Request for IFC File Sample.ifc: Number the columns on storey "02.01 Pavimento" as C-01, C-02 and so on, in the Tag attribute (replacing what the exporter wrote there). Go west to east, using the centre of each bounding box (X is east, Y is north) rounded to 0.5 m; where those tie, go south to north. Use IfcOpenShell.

First a look at what the model holds.

```python
import ifcopenshell
import ifcopenshell.util.element
import ifcopenshell.util.placement

model = ifcopenshell.open("IFC File Sample.ifc")
print(model.schema)
storey = next(s for s in model.by_type("IfcBuildingStorey") if s.Name == "02.01 Pavimento")
columns = [e for e in ifcopenshell.util.element.get_decomposition(storey) if e.is_a("IfcColumn")]
for e in sorted(columns, key=lambda e: e.id()):
    origin = ifcopenshell.util.placement.get_local_placement(e.ObjectPlacement)[:3, 3]
    print(e.id(), e.Tag, e.Name, origin.round(2) + 0.0, sep=" | ")
```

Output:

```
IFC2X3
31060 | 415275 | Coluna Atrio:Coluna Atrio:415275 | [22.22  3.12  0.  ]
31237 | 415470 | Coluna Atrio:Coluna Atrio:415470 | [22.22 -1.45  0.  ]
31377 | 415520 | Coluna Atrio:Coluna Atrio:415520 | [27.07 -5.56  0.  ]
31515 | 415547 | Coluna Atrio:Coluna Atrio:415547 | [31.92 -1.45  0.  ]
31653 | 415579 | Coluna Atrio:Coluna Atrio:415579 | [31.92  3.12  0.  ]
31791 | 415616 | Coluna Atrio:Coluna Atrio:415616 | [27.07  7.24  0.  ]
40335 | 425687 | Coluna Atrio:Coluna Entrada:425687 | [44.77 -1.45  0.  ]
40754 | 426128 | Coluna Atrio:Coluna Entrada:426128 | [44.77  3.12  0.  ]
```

```python
import ifcopenshell
import ifcopenshell.geom
import ifcopenshell.util.element
import ifcopenshell.util.shape

model = ifcopenshell.open("IFC File Sample.ifc")
settings = ifcopenshell.geom.settings()
settings.set("use-world-coords", True)


def centre(element):
    shape = ifcopenshell.geom.create_shape(settings, element)
    return ifcopenshell.util.shape.get_bbox_centroid(shape.geometry)


storey = next(s for s in model.by_type("IfcBuildingStorey") if s.Name == "02.01 Pavimento")
columns = [e for e in ifcopenshell.util.element.get_decomposition(storey) if e.is_a("IfcColumn")]

# Insertion points can sit at a corner or the storey origin, so sort by the geometry (in metres).
centres = {e: centre(e) for e in columns}
columns.sort(key=lambda e: (round(centres[e][0] / 0.5), centres[e][1]))

for i, e in enumerate(columns, start=1):
    number = f"C-{i:02d}"
    e.Tag = number
    print(e.id(), number)

model.write("IFC File Sample_edited.ifc")
```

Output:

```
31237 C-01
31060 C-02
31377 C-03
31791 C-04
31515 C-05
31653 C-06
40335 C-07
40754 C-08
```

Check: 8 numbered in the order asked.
